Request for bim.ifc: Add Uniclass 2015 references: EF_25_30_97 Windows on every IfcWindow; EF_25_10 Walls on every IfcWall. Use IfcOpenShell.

First a look at what the model holds.

```python
import ifcopenshell

model = ifcopenshell.open("bim.ifc")
print(model.schema)
print("classifications:", [c.Name for c in model.by_type("IfcClassification")])
for ifc_class in ("IfcDoor", "IfcRoof", "IfcStair", "IfcWall", "IfcWindow"):
    print(ifc_class, len(model.by_type(ifc_class)))
```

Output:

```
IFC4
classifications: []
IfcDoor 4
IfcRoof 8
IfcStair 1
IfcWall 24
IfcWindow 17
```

```python
import ifcopenshell
import ifcopenshell.api.classification

model = ifcopenshell.open("bim.ifc")

system = ifcopenshell.api.classification.add_classification(model, classification="Uniclass 2015")

codes = {
    "IfcWindow": ("EF_25_30_97", "Windows"),
    "IfcWall": ("EF_25_10", "Walls"),
}
for ifc_class, (code, name) in codes.items():
    products = model.by_type(ifc_class)
    ifcopenshell.api.classification.add_reference(
        model, products=products, classification=system, identification=code, name=name
    )
    print(code, len(products))

model.write("bim_v2.ifc")
```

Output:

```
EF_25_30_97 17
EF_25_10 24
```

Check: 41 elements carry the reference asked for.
